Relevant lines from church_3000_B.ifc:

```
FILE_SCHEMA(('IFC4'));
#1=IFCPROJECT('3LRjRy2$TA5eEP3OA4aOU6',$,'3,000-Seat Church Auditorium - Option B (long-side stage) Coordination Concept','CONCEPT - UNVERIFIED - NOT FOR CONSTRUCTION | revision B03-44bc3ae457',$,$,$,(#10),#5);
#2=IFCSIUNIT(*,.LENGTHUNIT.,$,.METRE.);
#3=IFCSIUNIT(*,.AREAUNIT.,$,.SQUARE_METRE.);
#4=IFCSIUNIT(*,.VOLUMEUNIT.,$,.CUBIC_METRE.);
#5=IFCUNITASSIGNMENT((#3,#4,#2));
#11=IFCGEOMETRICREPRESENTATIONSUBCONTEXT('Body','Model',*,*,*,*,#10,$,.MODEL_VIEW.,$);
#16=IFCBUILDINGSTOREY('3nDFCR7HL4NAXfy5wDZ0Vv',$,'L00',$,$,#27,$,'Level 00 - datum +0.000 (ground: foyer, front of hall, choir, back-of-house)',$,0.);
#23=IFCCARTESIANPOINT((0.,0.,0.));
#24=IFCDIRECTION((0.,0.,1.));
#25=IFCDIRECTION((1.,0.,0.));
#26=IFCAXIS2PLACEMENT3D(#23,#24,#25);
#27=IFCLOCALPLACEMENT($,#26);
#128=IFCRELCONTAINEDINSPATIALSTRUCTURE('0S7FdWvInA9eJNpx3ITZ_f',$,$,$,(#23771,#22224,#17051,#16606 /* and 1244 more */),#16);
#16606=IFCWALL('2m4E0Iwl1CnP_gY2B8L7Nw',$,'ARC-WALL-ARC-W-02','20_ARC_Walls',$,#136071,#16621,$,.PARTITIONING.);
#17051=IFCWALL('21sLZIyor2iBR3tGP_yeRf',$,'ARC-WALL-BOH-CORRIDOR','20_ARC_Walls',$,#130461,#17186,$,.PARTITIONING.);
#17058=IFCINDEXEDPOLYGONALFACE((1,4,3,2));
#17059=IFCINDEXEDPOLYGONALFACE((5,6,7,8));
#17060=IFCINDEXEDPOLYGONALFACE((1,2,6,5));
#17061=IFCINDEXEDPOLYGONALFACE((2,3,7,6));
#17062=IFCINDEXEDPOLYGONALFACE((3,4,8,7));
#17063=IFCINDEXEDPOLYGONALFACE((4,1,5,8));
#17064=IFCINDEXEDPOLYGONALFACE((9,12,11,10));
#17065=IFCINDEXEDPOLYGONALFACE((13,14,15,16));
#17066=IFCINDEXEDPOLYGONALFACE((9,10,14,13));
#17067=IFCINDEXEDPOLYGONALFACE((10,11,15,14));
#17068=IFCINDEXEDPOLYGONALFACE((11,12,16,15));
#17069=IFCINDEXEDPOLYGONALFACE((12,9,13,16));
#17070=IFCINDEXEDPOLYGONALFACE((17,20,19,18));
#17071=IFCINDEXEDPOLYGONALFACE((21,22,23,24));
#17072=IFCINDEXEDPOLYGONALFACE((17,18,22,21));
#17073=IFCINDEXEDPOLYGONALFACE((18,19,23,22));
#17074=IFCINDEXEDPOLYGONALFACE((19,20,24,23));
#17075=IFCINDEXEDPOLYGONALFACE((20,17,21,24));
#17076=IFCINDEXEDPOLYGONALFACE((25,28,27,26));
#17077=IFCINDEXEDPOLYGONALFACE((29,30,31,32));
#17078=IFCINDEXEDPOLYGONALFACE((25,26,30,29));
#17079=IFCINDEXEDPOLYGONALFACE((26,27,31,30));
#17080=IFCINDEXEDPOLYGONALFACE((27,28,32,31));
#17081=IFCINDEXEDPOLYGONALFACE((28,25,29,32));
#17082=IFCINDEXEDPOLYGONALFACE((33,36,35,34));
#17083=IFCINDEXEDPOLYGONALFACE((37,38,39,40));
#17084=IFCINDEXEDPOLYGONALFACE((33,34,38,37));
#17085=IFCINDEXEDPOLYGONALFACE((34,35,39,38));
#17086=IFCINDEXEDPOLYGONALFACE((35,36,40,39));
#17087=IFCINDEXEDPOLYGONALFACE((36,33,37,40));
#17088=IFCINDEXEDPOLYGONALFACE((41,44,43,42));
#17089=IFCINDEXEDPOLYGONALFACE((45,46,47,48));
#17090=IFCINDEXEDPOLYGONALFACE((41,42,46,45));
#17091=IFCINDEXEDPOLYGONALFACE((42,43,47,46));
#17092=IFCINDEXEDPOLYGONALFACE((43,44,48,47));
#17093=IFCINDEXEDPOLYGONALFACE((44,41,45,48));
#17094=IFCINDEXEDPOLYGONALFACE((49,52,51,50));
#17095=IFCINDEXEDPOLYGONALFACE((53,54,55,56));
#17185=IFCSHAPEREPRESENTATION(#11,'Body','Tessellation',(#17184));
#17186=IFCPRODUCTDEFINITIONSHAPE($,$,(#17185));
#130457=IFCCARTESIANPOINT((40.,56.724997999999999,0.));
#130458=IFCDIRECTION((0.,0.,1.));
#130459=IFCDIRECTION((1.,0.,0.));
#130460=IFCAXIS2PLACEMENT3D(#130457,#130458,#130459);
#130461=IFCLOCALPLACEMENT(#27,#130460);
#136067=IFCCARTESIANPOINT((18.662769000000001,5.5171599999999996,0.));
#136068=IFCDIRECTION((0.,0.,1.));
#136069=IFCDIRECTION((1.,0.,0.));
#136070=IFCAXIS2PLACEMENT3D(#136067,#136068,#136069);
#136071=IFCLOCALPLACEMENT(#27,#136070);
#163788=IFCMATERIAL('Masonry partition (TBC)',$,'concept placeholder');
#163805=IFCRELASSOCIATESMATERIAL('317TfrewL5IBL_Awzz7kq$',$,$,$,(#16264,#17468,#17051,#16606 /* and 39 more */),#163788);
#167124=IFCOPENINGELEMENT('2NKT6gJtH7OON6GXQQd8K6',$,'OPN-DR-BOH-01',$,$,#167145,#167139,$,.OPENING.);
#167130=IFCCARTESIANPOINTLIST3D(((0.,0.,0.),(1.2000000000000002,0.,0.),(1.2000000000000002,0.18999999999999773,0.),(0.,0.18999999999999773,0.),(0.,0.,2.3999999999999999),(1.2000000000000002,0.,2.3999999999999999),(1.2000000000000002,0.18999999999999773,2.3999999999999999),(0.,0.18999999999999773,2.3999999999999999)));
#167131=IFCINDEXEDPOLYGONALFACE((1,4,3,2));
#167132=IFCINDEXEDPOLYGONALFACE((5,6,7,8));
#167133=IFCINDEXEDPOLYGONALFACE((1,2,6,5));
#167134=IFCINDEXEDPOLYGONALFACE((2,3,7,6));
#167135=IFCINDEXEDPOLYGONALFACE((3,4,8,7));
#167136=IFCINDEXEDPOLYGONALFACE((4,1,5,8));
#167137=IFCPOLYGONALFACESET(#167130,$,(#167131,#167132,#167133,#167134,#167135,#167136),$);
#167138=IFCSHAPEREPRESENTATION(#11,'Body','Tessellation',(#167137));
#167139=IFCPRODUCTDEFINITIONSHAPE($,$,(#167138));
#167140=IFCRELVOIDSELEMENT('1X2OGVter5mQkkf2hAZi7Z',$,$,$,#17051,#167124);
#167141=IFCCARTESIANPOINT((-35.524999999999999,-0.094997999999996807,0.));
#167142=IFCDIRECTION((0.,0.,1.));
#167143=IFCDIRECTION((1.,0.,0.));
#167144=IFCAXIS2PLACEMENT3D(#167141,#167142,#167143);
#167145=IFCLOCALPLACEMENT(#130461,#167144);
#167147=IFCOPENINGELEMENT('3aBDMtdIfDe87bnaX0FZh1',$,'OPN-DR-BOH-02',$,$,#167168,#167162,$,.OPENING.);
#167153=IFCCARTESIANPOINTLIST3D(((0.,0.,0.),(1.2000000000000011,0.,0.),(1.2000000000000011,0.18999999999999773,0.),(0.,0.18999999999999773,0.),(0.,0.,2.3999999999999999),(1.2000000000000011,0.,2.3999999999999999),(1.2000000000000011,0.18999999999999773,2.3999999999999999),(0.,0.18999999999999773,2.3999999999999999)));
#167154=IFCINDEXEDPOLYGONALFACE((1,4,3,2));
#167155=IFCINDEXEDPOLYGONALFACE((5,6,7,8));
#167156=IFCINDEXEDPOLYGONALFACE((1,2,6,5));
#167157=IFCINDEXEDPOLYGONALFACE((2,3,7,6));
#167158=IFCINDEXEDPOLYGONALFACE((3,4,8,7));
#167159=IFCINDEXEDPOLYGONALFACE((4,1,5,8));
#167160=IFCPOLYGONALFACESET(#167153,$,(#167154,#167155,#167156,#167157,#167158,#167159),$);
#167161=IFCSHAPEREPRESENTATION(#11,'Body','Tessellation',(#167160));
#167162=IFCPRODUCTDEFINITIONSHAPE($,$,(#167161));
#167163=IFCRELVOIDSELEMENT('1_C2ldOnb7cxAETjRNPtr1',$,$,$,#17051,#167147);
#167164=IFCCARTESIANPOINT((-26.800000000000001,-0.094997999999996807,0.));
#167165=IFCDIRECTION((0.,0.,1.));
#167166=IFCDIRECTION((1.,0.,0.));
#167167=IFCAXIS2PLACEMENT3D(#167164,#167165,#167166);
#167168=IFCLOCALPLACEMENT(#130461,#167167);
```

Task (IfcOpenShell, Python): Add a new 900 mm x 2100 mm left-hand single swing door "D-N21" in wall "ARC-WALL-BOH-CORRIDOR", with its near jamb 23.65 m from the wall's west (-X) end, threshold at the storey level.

```python
import numpy as np
import ifcopenshell
import ifcopenshell.api.feature
import ifcopenshell.api.geometry
import ifcopenshell.api.root
import ifcopenshell.api.spatial
import ifcopenshell.geom
import ifcopenshell.util.element
import ifcopenshell.util.placement
import ifcopenshell.util.representation
import ifcopenshell.util.shape
import ifcopenshell.util.unit

model = ifcopenshell.open("church_3000_B.ifc")
unit_scale = ifcopenshell.util.unit.calculate_unit_scale(model)
settings = ifcopenshell.geom.settings()


def volume(element):
    """Net volume in cubic metres, openings subtracted."""
    shape = ifcopenshell.geom.create_shape(settings, element)
    return ifcopenshell.util.shape.get_volume(shape.geometry)


wall = model.by_guid("21sLZIyor2iBR3tGP_yeRf")
storey = ifcopenshell.util.element.get_container(wall, ifc_class="IfcBuildingStorey")
context = ifcopenshell.util.representation.get_context(model, "Model", "Body", "MODEL_VIEW")
before = volume(wall)

width, height, from_end, sill = 0.9, 2.1, 23.65, 0.0  # metres

# The wall runs along its own X axis, and the end named is its -X end.
wall_shape = ifcopenshell.geom.create_shape(settings, wall)
x, y, z = ifcopenshell.util.shape.get_vertices(wall_shape.geometry).T
start = x.min() + from_end
face, thickness = float(y.min()), float(y.max() - y.min())
wall_matrix = ifcopenshell.util.placement.get_local_placement(wall.ObjectPlacement)
level = ifcopenshell.util.placement.get_local_placement(storey.ObjectPlacement)[2, 3]


def in_wall(x, y):
    """Placement at x, y metres in the wall's axes, at sill height."""
    matrix = wall_matrix.copy()
    matrix[:, 3] = wall_matrix @ np.array([x / unit_scale, y / unit_scale, 0.0, 1.0])
    matrix[2, 3] = level + sill / unit_scale
    return matrix


# Opening: a box that overshoots both wall faces by 50 mm.
opening = ifcopenshell.api.root.create_entity(model, ifc_class="IfcOpeningElement", predefined_type="OPENING")
box = ifcopenshell.api.geometry.add_wall_representation(
    model, context=context, length=width, height=height, thickness=thickness + 0.1
)
ifcopenshell.api.geometry.assign_representation(model, product=opening, representation=box)
ifcopenshell.api.geometry.edit_object_placement(model, product=opening, matrix=in_wall(start, face - 0.05), is_si=False)
ifcopenshell.api.feature.add_feature(model, feature=opening, element=wall)

door = ifcopenshell.api.root.create_entity(model, ifc_class="IfcDoor", name="D-N21", predefined_type="DOOR")
door.OverallWidth, door.OverallHeight = width / unit_scale, height / unit_scale
door.OperationType = "SINGLE_SWING_LEFT"
body = ifcopenshell.api.geometry.add_door_representation(
    model,
    context=context,
    overall_width=door.OverallWidth,
    overall_height=door.OverallHeight,
    operation_type="SINGLE_SWING_LEFT",
    lining_properties={"LiningDepth": thickness / unit_scale, "ThresholdDepth": thickness / unit_scale},
)
ifcopenshell.api.geometry.assign_representation(model, product=door, representation=body)
ifcopenshell.api.spatial.assign_container(model, products=[door], relating_structure=storey)
ifcopenshell.api.feature.add_filling(model, opening=opening, element=door)

# The lining spans the wall, so the door starts at the wall face.
ifcopenshell.api.geometry.edit_object_placement(model, product=door, matrix=in_wall(start, face), is_si=False)

after = volume(wall)

print(f"wall volume {before:.3f} -> {after:.3f} m3")

model.write("church_3000_B-out.ifc")
```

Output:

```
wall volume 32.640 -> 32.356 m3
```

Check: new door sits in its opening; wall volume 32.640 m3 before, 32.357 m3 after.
